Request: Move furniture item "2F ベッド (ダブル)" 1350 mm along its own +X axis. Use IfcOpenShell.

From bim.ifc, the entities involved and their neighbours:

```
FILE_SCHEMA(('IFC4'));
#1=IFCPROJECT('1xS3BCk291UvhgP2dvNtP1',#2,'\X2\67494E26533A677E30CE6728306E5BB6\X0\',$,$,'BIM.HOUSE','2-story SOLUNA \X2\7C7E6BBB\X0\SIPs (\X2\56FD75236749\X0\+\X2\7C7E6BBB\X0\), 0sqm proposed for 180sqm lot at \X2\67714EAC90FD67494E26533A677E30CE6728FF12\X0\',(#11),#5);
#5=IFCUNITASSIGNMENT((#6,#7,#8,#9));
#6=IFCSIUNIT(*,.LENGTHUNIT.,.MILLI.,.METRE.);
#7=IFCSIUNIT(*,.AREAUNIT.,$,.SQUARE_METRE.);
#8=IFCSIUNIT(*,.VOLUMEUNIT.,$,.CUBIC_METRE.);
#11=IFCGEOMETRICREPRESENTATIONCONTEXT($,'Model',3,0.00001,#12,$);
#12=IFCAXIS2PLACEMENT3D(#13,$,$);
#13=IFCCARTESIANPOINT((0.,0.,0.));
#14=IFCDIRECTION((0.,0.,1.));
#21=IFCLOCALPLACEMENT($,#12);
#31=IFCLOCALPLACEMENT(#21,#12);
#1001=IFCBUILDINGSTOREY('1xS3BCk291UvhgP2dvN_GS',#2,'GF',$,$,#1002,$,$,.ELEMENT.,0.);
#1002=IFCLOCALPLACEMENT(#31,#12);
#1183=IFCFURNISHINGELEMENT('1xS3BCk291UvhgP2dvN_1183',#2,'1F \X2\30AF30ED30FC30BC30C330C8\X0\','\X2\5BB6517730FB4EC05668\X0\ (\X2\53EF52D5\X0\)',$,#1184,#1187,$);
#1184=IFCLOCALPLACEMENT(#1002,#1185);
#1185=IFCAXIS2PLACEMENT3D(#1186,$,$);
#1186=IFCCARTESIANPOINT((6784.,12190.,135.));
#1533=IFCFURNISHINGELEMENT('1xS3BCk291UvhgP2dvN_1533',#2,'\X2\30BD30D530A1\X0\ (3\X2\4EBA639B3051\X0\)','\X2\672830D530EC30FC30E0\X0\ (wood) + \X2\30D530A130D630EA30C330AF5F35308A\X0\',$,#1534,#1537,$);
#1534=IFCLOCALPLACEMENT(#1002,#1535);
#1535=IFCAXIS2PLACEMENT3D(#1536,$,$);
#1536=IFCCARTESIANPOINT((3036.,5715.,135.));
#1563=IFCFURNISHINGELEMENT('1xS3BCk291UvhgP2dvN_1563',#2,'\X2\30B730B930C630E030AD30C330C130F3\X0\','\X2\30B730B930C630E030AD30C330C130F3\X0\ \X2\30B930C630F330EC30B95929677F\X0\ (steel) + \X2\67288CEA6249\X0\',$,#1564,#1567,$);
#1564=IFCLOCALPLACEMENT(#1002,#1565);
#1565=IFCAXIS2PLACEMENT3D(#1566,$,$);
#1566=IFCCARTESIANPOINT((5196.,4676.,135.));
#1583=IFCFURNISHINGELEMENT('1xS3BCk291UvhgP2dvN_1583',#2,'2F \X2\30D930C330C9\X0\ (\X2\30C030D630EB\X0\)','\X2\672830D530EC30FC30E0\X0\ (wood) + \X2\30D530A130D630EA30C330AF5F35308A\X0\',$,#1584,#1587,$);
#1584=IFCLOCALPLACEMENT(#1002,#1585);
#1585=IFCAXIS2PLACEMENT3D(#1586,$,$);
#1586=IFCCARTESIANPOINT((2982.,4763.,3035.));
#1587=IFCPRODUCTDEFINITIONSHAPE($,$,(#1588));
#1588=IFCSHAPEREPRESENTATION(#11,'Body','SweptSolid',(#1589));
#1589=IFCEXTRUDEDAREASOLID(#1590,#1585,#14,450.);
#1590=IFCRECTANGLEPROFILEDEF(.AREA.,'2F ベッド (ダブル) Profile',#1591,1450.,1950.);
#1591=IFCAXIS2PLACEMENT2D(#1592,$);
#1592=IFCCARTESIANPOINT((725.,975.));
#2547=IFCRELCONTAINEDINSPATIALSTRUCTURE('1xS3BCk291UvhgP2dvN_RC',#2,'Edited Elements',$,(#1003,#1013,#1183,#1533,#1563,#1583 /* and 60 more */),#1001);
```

```python
import ifcopenshell
import ifcopenshell.api.geometry
import ifcopenshell.util.placement
import ifcopenshell.util.unit

model = ifcopenshell.open("bim.ifc")
unit_scale = ifcopenshell.util.unit.calculate_unit_scale(model)

item = model.by_guid("1xS3BCk291UvhgP2dvN_1583")
matrix = ifcopenshell.util.placement.get_local_placement(item.ObjectPlacement)
matrix[:3, 3] += matrix[:3, 0] * 1.35 / unit_scale
ifcopenshell.api.geometry.edit_object_placement(model, product=item, matrix=matrix, is_si=False)

print(ifcopenshell.util.placement.get_local_placement(item.ObjectPlacement).round(3) + 0.0)

model.write("bim-out.ifc")
```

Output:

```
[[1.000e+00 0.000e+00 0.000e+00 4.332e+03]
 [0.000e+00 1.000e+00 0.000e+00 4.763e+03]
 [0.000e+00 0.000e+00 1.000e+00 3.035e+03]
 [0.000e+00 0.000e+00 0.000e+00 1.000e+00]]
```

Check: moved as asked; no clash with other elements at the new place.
